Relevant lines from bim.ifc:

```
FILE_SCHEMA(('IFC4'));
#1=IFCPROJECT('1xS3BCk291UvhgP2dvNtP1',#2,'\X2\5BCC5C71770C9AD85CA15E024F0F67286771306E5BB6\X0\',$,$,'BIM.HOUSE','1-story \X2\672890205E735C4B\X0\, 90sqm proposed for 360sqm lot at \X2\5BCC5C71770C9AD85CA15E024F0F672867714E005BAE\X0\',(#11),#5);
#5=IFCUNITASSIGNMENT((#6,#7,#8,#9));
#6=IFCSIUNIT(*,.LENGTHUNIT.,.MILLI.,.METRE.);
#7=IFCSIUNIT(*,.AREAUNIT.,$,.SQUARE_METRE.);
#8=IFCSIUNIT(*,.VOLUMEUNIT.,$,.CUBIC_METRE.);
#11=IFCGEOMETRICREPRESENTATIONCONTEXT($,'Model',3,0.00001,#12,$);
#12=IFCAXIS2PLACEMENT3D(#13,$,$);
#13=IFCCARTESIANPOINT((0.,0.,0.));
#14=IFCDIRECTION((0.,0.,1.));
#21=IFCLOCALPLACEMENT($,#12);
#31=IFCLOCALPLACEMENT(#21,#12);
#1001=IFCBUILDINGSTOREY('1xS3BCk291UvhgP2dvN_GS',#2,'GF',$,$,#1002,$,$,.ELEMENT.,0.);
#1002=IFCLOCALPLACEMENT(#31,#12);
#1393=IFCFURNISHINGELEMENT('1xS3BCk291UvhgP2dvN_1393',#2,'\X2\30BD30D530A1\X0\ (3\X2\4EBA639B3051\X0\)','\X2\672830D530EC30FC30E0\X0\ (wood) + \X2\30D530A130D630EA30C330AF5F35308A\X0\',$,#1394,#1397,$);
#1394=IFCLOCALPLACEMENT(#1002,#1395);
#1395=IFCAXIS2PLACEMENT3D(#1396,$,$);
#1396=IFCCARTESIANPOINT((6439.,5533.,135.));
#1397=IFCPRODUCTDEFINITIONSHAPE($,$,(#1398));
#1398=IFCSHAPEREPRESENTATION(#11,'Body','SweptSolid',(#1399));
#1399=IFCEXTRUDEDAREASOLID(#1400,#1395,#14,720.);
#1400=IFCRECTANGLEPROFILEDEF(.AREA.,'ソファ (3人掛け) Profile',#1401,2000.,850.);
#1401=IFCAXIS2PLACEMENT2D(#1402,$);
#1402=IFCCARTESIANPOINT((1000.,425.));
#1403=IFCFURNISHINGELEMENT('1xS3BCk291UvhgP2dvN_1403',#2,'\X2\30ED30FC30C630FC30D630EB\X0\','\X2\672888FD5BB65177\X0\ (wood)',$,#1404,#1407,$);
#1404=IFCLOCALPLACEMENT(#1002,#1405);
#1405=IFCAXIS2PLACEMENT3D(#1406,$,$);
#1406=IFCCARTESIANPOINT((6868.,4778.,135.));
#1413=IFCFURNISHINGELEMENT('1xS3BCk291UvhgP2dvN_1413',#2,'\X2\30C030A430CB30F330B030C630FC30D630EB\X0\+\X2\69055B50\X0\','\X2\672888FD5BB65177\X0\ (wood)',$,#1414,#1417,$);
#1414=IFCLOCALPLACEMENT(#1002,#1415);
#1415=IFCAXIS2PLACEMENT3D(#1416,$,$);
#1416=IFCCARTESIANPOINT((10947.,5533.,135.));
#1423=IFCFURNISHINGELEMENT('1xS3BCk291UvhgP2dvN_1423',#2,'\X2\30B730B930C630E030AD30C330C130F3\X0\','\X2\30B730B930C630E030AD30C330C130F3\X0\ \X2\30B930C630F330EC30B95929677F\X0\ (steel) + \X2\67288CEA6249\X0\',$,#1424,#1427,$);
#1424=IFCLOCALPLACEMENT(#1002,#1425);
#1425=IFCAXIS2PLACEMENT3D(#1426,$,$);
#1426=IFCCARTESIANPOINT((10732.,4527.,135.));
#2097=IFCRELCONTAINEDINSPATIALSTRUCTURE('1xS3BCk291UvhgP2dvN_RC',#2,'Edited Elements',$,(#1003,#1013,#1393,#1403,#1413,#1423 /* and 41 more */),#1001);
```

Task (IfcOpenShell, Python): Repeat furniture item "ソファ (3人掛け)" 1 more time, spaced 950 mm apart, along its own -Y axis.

```python
import ifcopenshell
import ifcopenshell.api.geometry
import ifcopenshell.api.root
import ifcopenshell.util.element
import ifcopenshell.util.placement
import ifcopenshell.util.unit

model = ifcopenshell.open("bim.ifc")
unit_scale = ifcopenshell.util.unit.calculate_unit_scale(model)


def reuse_history(source, copy):
    """copy_class also copies each property set's owner history, people and application; keep the originals."""
    for rel in copy.IsDefinedBy:
        if rel.is_a("IfcRelDefinesByProperties") and (history := rel.RelatingPropertyDefinition.OwnerHistory):
            rel.RelatingPropertyDefinition.OwnerHistory = source.OwnerHistory
            ifcopenshell.util.element.remove_deep2(model, history)


source = model.by_guid("1xS3BCk291UvhgP2dvN_1393")
base = ifcopenshell.util.placement.get_local_placement(source.ObjectPlacement)
step = -base[:3, 1] * 0.95 / unit_scale

for i in range(1, 2):
    copy = ifcopenshell.api.root.copy_class(model, product=source)
    copy.Representation = ifcopenshell.util.element.copy_deep(
        model, source.Representation, exclude=["IfcGeometricRepresentationContext", "IfcRepresentationMap"]
    )
    reuse_history(source, copy)
    matrix = base.copy()
    matrix[:3, 3] += i * step
    print("added at", matrix[:3, 3].round(3) + 0.0)
    ifcopenshell.api.geometry.edit_object_placement(model, product=copy, matrix=matrix, is_si=False)

model.write("bim_v2.ifc")
```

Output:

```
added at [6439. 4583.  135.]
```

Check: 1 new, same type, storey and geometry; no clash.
